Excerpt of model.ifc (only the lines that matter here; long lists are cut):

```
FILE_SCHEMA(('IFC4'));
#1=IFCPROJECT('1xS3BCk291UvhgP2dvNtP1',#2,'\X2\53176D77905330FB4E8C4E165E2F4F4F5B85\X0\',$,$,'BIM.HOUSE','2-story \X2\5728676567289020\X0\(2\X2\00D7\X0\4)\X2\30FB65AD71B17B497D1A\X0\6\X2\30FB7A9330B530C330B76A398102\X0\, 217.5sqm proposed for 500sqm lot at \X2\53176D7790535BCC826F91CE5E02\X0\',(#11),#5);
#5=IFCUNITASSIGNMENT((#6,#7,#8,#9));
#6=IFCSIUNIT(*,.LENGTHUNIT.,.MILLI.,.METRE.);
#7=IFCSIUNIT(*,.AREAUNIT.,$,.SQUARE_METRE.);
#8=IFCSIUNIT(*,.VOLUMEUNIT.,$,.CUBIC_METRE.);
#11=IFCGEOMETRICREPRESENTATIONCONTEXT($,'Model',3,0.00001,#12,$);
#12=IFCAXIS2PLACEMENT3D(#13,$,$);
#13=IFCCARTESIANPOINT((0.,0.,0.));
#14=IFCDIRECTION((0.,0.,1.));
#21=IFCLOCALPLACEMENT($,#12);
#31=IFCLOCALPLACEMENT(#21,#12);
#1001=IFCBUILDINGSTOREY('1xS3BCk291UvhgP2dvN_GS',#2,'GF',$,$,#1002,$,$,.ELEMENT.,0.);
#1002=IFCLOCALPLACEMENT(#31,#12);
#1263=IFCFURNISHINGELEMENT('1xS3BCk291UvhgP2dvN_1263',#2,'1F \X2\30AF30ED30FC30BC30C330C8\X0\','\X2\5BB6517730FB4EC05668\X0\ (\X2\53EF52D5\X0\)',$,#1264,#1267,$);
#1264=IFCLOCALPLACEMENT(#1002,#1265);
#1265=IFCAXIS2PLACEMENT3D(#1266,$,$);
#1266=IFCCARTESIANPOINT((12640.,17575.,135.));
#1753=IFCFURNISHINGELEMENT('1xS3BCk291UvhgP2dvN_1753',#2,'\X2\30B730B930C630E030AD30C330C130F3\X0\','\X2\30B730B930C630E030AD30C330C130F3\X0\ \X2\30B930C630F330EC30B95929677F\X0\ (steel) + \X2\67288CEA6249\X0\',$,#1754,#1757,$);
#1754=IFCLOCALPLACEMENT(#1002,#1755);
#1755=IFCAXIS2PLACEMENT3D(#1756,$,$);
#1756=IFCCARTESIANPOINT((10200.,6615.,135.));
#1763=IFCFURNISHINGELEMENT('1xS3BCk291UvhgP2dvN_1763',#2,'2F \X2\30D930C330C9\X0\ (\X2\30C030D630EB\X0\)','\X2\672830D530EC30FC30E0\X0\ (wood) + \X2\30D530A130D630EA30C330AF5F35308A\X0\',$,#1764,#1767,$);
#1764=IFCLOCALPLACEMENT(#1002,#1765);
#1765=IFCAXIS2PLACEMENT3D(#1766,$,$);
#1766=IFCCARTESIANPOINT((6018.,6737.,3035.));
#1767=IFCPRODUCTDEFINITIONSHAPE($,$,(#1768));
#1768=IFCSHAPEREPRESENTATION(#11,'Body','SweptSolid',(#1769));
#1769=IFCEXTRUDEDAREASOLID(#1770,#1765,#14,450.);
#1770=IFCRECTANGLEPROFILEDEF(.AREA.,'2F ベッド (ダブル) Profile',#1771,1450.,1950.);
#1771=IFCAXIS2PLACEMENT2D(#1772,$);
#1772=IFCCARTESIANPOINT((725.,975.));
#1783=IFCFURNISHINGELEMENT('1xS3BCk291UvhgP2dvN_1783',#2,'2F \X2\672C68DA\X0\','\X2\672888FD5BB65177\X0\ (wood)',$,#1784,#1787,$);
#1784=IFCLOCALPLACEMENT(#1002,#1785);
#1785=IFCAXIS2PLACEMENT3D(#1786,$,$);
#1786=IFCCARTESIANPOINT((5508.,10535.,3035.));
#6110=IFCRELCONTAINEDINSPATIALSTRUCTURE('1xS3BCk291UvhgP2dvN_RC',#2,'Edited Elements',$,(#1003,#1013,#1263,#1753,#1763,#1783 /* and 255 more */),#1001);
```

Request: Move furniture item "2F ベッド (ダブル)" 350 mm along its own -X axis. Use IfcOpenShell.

```python
import ifcopenshell
import ifcopenshell.api.geometry
import ifcopenshell.util.placement

model = ifcopenshell.open("model.ifc")

item = model.by_guid("1xS3BCk291UvhgP2dvN_1763")
matrix = ifcopenshell.util.placement.get_local_placement(item.ObjectPlacement)
matrix[:3, 3] -= matrix[:3, 0] * 350.0
ifcopenshell.api.geometry.edit_object_placement(model, product=item, matrix=matrix, is_si=False)

print(ifcopenshell.util.placement.get_local_placement(item.ObjectPlacement).round(3) + 0.0)

model.write("model_v2.ifc")
```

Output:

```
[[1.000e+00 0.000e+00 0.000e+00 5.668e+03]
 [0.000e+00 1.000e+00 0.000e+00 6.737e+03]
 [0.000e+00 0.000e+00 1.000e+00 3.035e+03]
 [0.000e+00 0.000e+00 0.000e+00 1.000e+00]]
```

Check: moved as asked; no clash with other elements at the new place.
